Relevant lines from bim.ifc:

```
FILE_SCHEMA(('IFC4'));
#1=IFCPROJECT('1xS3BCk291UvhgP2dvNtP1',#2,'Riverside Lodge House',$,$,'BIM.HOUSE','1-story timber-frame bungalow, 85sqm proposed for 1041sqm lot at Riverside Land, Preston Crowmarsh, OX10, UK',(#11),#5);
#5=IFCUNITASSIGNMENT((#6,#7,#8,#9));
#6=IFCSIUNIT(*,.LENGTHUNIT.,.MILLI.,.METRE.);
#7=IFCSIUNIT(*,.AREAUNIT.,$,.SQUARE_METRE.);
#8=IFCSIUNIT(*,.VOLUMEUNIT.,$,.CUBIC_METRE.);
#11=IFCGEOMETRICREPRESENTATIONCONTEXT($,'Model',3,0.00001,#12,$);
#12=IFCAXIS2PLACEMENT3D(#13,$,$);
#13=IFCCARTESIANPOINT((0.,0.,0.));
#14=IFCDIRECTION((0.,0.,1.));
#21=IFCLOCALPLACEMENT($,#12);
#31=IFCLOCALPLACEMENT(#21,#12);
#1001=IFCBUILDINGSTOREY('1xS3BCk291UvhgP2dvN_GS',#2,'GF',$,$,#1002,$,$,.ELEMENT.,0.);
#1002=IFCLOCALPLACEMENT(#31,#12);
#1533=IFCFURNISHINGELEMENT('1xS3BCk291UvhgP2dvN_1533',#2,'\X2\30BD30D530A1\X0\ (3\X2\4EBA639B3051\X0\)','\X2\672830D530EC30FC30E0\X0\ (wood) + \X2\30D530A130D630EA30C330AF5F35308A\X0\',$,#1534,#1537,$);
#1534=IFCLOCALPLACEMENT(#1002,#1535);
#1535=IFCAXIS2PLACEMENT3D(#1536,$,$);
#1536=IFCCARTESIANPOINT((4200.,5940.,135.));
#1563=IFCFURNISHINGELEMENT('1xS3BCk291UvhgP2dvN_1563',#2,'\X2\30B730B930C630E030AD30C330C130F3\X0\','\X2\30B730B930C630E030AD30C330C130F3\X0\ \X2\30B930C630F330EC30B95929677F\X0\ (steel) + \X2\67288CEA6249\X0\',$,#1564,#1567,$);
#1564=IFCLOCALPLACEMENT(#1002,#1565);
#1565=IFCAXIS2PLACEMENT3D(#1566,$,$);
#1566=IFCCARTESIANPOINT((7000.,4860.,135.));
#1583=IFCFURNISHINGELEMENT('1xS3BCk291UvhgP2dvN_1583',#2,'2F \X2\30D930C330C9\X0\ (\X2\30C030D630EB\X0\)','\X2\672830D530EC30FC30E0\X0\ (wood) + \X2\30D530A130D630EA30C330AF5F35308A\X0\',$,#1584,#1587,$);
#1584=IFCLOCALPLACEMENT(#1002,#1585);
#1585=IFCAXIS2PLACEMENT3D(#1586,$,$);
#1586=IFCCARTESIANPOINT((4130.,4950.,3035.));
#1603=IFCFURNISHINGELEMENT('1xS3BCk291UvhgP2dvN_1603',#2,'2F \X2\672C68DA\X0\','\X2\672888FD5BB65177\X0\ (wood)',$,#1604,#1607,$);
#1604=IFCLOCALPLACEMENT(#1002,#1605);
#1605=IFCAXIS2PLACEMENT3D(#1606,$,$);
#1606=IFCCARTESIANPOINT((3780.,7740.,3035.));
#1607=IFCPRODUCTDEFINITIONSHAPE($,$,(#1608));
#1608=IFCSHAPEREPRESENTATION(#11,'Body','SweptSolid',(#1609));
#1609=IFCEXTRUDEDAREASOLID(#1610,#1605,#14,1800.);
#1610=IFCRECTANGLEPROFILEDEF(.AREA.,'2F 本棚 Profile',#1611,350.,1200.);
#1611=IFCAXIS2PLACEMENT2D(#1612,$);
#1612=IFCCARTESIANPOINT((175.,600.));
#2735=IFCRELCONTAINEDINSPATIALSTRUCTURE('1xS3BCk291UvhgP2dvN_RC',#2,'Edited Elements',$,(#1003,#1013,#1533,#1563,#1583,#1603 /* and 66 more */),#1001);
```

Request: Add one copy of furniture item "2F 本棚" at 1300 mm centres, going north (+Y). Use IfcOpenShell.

```python
import numpy as np
import ifcopenshell
import ifcopenshell.api.geometry
import ifcopenshell.api.root
import ifcopenshell.util.element
import ifcopenshell.util.placement
import ifcopenshell.util.unit

model = ifcopenshell.open("bim.ifc")
unit_scale = ifcopenshell.util.unit.calculate_unit_scale(model)


def reuse_history(source, copy):
    """copy_class also copies each property set's owner history, people and application; keep the originals."""
    for rel in copy.IsDefinedBy:
        if rel.is_a("IfcRelDefinesByProperties") and (history := rel.RelatingPropertyDefinition.OwnerHistory):
            rel.RelatingPropertyDefinition.OwnerHistory = source.OwnerHistory
            ifcopenshell.util.element.remove_deep2(model, history)


source = model.by_guid("1xS3BCk291UvhgP2dvN_1603")
base = ifcopenshell.util.placement.get_local_placement(source.ObjectPlacement)
step = np.array([0.0, 1.0, 0.0]) * 1.3 / unit_scale

for i in range(1, 2):
    copy = ifcopenshell.api.root.copy_class(model, product=source)
    copy.Representation = ifcopenshell.util.element.copy_deep(
        model, source.Representation, exclude=["IfcGeometricRepresentationContext", "IfcRepresentationMap"]
    )
    reuse_history(source, copy)
    matrix = base.copy()
    matrix[:3, 3] += i * step
    print("added at", matrix[:3, 3].round(3) + 0.0)
    ifcopenshell.api.geometry.edit_object_placement(model, product=copy, matrix=matrix, is_si=False)

model.write("bim-out.ifc")
```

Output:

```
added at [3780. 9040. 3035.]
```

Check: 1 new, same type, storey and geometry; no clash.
